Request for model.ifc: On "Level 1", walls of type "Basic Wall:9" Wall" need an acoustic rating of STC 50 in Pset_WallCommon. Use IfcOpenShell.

First a look at what the model holds.

```python
import ifcopenshell
import ifcopenshell.util.element

model = ifcopenshell.open("model.ifc")
print(model.schema)
storey = next(s for s in model.by_type("IfcBuildingStorey") if s.Name == "Level 1")
walls = [e for e in ifcopenshell.util.element.get_decomposition(storey) if e.is_a("IfcWall")]
seen = {}
for e in walls:
    element_type = ifcopenshell.util.element.get_type(e)
    key = (element_type.Name if element_type != e and element_type else None, ifcopenshell.util.element.get_pset(e, "Pset_WallCommon", "AcousticRating"))
    seen[key] = seen.get(key, 0) + 1
for (name, value), count in sorted(seen.items(), key=str):
    print(count, "x", name, "|", value)
```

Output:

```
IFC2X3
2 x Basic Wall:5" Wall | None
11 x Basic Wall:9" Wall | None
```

```python
import ifcopenshell
import ifcopenshell.api.pset
import ifcopenshell.util.element

model = ifcopenshell.open("model.ifc")

storey = next(s for s in model.by_type("IfcBuildingStorey") if s.Name == "Level 1")
walls = [e for e in ifcopenshell.util.element.get_decomposition(storey) if e.is_a("IfcWall")]

count = 0
for e in walls:
    element_type = ifcopenshell.util.element.get_type(e)
    if element_type in (None, e) or element_type.Name != 'Basic Wall:9" Wall':
        continue
    # add_pset returns the element's existing set when there is one.
    pset = ifcopenshell.api.pset.add_pset(model, product=e, name="Pset_WallCommon")
    ifcopenshell.api.pset.edit_pset(model, pset=pset, properties={"AcousticRating": "STC 50"})
    count += 1

print(count, "walls updated")

model.write("model_edited.ifc")
```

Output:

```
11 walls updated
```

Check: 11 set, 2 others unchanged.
